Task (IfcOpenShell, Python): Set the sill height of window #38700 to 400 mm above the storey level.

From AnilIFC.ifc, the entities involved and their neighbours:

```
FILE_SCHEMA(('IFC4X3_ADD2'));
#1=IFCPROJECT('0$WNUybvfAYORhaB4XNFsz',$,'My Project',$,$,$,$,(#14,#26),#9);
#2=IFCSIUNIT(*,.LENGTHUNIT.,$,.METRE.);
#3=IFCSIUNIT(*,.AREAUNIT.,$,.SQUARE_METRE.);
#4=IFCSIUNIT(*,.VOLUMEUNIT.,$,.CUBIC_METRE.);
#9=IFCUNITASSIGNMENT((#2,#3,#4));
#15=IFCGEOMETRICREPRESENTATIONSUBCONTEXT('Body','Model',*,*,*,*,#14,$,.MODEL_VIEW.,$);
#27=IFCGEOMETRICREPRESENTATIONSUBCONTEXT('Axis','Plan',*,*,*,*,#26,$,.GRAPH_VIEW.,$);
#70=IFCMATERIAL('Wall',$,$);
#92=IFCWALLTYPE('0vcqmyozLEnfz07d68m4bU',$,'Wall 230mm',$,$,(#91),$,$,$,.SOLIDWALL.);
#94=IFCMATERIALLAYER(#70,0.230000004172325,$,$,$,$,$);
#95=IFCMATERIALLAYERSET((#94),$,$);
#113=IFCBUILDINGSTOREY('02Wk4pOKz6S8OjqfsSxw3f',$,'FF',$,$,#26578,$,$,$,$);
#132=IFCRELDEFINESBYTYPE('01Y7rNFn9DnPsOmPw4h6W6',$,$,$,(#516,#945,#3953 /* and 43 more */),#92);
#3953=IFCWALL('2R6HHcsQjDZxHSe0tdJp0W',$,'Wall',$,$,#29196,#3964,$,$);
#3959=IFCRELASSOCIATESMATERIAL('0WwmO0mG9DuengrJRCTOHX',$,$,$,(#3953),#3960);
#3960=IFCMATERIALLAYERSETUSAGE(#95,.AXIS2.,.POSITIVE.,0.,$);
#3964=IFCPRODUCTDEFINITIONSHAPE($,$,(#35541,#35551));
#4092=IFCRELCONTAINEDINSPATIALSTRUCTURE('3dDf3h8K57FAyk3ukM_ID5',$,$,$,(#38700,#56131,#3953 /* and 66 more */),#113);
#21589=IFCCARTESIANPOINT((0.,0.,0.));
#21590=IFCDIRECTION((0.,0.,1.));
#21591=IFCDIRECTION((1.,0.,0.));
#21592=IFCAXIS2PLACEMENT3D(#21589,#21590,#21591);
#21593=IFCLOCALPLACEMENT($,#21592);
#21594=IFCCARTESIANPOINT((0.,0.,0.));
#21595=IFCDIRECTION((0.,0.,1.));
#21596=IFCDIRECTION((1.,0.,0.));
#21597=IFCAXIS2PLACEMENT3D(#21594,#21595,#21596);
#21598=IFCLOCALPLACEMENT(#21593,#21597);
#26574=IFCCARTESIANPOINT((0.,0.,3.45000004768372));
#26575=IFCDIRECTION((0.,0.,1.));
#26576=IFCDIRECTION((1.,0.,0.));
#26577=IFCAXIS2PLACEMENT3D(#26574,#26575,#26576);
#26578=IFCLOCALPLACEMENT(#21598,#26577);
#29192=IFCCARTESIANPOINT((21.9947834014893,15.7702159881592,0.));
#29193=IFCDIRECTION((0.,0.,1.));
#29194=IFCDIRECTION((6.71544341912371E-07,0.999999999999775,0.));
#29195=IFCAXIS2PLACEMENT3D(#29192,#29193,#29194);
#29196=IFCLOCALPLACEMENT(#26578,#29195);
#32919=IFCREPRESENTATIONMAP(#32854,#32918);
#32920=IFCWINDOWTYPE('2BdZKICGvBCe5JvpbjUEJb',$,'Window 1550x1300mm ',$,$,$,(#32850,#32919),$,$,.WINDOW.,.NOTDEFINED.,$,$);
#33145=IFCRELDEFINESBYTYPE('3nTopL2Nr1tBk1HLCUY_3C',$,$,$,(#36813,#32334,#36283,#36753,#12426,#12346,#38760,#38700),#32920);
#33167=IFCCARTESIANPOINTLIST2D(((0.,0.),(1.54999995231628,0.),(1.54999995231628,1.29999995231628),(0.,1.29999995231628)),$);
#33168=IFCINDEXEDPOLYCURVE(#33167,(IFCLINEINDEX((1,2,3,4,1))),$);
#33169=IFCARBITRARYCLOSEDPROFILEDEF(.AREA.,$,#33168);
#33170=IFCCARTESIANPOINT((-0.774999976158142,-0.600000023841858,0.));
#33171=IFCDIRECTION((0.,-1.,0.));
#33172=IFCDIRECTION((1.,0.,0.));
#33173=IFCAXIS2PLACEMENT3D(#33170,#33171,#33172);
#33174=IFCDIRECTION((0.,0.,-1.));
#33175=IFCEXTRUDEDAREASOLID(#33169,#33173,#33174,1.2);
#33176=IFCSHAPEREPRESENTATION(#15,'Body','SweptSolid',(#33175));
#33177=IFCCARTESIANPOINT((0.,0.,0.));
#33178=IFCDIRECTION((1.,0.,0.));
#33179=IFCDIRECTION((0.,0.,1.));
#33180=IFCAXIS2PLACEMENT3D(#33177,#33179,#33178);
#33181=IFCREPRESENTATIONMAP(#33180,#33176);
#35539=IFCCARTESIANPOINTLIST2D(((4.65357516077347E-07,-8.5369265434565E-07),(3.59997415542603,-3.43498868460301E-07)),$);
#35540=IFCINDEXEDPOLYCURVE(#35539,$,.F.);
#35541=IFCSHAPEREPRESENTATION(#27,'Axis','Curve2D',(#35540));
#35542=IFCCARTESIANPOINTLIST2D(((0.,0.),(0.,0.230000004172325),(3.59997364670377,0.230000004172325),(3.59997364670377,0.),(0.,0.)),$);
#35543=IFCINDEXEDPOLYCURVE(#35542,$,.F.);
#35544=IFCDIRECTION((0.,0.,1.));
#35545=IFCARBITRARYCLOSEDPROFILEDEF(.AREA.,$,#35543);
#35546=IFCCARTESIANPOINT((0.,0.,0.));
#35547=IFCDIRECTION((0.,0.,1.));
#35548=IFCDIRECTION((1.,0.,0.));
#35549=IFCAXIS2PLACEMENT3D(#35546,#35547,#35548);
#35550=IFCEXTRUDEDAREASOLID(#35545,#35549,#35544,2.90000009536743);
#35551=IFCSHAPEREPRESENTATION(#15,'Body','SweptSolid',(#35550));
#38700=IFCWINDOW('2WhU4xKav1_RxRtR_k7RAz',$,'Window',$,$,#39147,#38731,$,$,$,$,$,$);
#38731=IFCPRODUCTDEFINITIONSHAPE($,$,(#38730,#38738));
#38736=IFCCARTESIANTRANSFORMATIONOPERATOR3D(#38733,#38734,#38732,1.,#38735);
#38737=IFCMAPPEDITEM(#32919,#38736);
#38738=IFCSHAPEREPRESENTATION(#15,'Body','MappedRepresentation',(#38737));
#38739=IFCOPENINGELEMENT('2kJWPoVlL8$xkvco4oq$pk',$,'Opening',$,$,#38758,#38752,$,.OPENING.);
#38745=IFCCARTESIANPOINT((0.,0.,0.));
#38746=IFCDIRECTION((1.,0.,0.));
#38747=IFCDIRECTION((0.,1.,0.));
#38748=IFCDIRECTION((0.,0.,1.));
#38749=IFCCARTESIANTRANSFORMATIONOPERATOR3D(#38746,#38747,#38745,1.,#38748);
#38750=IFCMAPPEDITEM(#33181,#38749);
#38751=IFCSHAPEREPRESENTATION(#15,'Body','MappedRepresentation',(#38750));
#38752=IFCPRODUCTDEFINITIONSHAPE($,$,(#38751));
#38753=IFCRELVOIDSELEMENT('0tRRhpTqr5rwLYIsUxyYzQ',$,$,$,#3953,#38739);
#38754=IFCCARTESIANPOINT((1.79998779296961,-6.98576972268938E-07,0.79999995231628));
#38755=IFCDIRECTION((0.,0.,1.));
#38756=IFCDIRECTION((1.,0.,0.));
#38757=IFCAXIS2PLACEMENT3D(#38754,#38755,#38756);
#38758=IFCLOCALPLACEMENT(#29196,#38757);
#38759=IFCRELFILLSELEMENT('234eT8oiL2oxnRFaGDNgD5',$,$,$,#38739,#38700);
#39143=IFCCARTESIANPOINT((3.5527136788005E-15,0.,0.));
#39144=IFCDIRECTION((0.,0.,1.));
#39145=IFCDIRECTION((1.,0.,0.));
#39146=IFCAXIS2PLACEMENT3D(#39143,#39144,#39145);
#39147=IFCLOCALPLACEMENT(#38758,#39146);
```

```python
import numpy as np
import ifcopenshell
import ifcopenshell.api.geometry
import ifcopenshell.geom
import ifcopenshell.util.element
import ifcopenshell.util.placement
import ifcopenshell.util.shape
import ifcopenshell.util.unit

model = ifcopenshell.open("AnilIFC.ifc")
unit_scale = ifcopenshell.util.unit.calculate_unit_scale(model)

window = model.by_guid("2WhU4xKav1_RxRtR_k7RAz")
opening = window.FillsVoids[0].RelatingOpeningElement
storey = ifcopenshell.util.element.get_container(window, ifc_class="IfcBuildingStorey")
level = ifcopenshell.util.placement.get_local_placement(storey.ObjectPlacement)[2, 3]

# The opening's origin need not be at the sill, so measure its lowest point.
shape = ifcopenshell.geom.create_shape(ifcopenshell.geom.settings(), opening)
bottom = ifcopenshell.util.shape.get_shape_bottom_elevation(shape, shape.geometry) / unit_scale
dz = level + 0.4 - bottom

shift = np.array([0.0, 0.0, dz])
# The window is placed relative to its opening, so it follows when the opening moves.
matrix = ifcopenshell.util.placement.get_local_placement(opening.ObjectPlacement)
matrix[:3, 3] += shift
ifcopenshell.api.geometry.edit_object_placement(
    model, product=opening, matrix=matrix, is_si=False, should_transform_children=True
)

print(f"moved by {dz * unit_scale:+.3f} m")

model.write("AnilIFC-out.ifc")
```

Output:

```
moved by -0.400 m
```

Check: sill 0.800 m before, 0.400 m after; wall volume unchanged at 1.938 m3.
